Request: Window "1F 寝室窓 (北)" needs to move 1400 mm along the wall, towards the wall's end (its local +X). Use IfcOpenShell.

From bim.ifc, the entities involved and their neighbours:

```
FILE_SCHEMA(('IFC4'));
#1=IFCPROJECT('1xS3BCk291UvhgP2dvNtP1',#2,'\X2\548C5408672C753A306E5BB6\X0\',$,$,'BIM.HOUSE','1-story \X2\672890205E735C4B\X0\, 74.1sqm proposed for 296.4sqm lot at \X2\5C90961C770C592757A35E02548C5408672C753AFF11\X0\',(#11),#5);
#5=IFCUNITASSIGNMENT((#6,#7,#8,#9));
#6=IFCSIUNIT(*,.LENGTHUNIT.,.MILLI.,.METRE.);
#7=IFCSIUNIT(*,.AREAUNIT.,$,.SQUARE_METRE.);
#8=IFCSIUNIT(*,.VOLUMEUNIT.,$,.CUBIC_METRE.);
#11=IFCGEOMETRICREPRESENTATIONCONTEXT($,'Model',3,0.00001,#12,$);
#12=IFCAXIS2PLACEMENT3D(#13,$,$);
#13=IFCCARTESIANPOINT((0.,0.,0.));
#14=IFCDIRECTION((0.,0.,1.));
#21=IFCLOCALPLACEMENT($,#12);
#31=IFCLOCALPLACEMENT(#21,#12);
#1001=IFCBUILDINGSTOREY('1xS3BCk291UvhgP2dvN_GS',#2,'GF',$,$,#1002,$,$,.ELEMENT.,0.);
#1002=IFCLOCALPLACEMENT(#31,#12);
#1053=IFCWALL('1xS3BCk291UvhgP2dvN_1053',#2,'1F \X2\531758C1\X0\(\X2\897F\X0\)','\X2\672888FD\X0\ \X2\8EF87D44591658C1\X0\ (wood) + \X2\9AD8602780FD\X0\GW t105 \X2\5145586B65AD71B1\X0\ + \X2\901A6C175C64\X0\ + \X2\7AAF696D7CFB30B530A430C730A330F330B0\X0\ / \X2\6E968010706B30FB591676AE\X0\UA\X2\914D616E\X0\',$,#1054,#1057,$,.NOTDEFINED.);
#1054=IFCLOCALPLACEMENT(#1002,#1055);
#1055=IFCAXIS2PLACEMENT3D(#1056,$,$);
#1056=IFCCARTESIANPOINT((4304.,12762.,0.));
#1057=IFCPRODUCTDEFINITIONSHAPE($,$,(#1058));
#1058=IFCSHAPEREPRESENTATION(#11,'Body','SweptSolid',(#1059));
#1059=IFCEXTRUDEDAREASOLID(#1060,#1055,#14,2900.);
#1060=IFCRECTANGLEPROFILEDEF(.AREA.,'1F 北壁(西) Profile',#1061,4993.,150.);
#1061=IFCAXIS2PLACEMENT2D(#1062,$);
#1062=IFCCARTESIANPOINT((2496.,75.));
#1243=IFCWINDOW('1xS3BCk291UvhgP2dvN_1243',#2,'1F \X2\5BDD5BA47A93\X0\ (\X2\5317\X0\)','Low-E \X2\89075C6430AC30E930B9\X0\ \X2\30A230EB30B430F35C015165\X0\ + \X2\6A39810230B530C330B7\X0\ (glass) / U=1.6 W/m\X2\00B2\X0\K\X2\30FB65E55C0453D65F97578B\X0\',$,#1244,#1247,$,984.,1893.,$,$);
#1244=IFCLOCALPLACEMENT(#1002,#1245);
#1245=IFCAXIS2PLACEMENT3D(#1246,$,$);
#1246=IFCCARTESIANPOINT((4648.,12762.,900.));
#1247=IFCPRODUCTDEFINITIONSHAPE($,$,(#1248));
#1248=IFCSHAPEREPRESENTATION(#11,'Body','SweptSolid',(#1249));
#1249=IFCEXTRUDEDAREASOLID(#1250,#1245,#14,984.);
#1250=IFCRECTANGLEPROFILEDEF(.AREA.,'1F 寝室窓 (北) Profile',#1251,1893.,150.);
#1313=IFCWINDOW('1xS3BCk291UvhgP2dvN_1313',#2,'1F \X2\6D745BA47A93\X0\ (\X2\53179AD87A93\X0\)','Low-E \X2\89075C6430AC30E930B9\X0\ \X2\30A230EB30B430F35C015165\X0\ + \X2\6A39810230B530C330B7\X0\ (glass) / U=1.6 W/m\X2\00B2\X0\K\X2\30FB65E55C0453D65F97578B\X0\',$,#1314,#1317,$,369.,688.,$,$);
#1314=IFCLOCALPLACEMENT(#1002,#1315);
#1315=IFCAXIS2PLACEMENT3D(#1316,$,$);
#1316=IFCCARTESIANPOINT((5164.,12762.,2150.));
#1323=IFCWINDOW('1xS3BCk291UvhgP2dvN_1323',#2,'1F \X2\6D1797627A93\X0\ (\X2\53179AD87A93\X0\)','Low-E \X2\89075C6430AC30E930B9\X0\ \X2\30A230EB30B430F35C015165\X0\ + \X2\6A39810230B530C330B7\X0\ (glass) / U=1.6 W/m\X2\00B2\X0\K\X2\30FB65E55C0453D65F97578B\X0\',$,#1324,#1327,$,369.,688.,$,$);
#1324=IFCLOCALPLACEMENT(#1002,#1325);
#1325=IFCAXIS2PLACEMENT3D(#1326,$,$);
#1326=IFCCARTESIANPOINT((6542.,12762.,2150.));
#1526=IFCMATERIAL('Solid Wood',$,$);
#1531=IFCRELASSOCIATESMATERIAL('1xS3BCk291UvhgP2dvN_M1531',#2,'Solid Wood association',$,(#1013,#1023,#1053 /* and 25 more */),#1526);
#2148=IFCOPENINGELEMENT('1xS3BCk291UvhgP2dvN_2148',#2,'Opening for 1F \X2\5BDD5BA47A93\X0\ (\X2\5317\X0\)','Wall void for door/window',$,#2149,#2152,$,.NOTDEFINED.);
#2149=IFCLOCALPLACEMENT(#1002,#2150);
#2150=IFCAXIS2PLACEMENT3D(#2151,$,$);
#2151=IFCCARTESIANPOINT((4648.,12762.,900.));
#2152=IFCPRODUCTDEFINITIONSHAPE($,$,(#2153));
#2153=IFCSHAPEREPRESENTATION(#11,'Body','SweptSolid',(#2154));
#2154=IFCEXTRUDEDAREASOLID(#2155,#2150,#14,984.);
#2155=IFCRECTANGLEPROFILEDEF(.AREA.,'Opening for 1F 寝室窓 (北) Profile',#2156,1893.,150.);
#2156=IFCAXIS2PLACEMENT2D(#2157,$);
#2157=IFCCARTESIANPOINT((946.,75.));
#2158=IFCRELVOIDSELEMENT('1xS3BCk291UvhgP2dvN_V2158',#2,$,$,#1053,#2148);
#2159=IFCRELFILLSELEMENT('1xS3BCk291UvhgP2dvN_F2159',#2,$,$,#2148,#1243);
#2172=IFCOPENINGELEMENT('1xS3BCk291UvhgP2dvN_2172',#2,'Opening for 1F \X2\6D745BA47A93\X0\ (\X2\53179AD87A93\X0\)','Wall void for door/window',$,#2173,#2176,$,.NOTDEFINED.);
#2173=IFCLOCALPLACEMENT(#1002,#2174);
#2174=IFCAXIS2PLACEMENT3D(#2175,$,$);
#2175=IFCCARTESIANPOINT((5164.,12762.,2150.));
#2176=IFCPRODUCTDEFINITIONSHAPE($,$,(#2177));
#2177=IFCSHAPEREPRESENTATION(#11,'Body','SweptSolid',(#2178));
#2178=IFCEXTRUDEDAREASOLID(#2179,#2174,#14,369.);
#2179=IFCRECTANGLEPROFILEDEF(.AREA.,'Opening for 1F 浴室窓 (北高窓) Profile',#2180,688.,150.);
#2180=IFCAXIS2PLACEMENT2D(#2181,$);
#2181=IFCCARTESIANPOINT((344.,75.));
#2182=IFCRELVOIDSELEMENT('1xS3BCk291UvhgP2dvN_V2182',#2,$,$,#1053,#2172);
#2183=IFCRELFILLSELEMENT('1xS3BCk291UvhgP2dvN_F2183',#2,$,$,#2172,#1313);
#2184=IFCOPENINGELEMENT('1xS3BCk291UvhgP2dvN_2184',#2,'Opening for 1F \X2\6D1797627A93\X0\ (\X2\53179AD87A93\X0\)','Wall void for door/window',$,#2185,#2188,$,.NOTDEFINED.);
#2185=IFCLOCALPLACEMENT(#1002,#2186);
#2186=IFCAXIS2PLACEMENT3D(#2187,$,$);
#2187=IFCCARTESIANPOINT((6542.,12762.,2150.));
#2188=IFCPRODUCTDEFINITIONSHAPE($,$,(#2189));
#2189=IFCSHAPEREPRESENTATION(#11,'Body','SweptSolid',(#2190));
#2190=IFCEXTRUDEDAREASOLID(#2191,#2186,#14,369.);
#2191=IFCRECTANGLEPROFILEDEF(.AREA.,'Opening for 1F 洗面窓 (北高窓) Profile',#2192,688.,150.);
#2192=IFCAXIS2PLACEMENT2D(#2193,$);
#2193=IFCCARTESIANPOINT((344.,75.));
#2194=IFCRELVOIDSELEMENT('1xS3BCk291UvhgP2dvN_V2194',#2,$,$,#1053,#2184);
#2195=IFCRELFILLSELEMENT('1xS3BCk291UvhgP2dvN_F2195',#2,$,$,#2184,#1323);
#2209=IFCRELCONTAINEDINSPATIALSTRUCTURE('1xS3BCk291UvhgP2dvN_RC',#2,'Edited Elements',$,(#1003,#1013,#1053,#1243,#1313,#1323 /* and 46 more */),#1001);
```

```python
import ifcopenshell
import ifcopenshell.api.geometry
import ifcopenshell.util.placement
import ifcopenshell.util.unit

model = ifcopenshell.open("bim.ifc")
unit_scale = ifcopenshell.util.unit.calculate_unit_scale(model)

window = model.by_id(1243)
opening = window.FillsVoids[0].RelatingOpeningElement
wall = opening.VoidsElements[0].RelatingBuildingElement

wall_matrix = ifcopenshell.util.placement.get_local_placement(wall.ObjectPlacement)
shift = wall_matrix[:3, 0] * 1.4 / unit_scale
before = ifcopenshell.util.placement.get_local_placement(window.ObjectPlacement)[:3, 3].copy()

# The window is not placed relative to its opening, so move both.
for product in (opening, window):
    matrix = ifcopenshell.util.placement.get_local_placement(product.ObjectPlacement)
    matrix[:3, 3] += shift
    ifcopenshell.api.geometry.edit_object_placement(model, product=product, matrix=matrix, is_si=False)

after = ifcopenshell.util.placement.get_local_placement(window.ObjectPlacement)[:3, 3]
print("window moved by", (after - before).round(3) + 0.0)

model.write("bim_v2.ifc")
```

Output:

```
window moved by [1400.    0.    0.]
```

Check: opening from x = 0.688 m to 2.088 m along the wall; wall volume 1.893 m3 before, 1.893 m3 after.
